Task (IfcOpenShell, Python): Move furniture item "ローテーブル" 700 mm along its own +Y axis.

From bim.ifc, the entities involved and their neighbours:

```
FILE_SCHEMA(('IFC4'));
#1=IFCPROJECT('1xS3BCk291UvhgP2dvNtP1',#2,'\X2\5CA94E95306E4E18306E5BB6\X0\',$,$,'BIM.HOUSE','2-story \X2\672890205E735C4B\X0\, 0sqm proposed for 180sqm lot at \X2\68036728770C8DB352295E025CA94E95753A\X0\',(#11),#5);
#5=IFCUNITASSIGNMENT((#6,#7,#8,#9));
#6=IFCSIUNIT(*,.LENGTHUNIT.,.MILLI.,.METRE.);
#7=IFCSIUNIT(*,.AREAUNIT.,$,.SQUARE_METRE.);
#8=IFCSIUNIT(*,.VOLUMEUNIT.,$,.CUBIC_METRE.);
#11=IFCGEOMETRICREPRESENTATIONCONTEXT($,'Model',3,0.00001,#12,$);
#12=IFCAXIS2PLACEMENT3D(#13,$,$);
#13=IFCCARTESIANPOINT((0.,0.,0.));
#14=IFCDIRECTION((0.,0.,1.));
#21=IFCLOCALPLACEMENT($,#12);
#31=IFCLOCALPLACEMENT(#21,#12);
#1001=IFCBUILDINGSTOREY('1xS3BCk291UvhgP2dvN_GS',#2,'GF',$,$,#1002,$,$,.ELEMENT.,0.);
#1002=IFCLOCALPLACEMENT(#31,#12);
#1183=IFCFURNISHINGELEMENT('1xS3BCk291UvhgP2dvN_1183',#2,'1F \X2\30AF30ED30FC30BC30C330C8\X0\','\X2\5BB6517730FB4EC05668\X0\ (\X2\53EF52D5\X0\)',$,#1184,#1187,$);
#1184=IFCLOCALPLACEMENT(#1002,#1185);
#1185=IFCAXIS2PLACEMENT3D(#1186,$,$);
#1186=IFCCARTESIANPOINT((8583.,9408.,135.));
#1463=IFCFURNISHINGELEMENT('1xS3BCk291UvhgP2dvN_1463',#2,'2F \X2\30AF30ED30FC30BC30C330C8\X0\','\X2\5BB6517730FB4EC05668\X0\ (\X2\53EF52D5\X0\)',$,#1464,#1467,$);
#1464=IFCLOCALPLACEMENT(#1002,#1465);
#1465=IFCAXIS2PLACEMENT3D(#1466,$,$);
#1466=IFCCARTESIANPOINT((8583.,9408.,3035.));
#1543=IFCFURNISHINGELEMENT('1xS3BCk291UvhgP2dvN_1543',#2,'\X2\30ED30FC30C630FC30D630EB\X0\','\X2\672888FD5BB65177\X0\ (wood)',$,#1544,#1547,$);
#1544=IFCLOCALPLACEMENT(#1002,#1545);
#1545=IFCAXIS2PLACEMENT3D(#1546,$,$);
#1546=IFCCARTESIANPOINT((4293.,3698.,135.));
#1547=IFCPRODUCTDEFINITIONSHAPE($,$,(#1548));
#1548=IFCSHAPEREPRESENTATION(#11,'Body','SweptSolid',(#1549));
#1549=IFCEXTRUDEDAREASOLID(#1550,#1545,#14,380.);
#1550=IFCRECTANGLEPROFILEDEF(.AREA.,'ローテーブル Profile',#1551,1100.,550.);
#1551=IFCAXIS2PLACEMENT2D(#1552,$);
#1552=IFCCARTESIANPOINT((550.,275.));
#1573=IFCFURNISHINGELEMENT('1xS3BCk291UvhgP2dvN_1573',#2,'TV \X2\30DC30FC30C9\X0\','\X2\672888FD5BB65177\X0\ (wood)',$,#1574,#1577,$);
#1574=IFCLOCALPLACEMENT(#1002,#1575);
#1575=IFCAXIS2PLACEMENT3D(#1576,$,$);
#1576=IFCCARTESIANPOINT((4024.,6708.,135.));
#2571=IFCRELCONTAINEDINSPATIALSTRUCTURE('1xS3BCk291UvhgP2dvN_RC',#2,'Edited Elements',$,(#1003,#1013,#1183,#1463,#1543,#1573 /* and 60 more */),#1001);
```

```python
import ifcopenshell
import ifcopenshell.api.geometry
import ifcopenshell.util.placement
import ifcopenshell.util.unit

model = ifcopenshell.open("bim.ifc")
unit_scale = ifcopenshell.util.unit.calculate_unit_scale(model)

item = model.by_guid("1xS3BCk291UvhgP2dvN_1543")
matrix = ifcopenshell.util.placement.get_local_placement(item.ObjectPlacement)
matrix[:3, 3] += matrix[:3, 1] * 0.7 / unit_scale
ifcopenshell.api.geometry.edit_object_placement(model, product=item, matrix=matrix, is_si=False)

print(ifcopenshell.util.placement.get_local_placement(item.ObjectPlacement).round(3) + 0.0)

model.write("bim_edited.ifc")
```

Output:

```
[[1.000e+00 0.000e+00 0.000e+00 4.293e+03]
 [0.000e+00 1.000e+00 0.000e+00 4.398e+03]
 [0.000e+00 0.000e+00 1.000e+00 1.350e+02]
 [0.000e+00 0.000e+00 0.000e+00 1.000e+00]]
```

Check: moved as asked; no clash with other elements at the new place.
